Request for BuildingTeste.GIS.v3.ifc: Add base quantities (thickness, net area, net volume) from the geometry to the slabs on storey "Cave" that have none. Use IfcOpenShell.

First a look at what the model holds.

```python
import ifcopenshell
import ifcopenshell.util.element
import ifcopenshell.util.unit

model = ifcopenshell.open("BuildingTeste.GIS.v3.ifc")
print(model.schema)
for unit_type in ("LENGTHUNIT", "AREAUNIT", "VOLUMEUNIT"):
    print(unit_type, ifcopenshell.util.unit.calculate_unit_scale(model, unit_type))
storey = next(s for s in model.by_type("IfcBuildingStorey") if s.Name == "Cave")
slabs = [e for e in ifcopenshell.util.element.get_decomposition(storey) if e.is_a("IfcSlab")]
for e in sorted(slabs, key=lambda e: e.id()):
    print(e.id(), e.is_a(), e.Name, list(ifcopenshell.util.element.get_psets(e, qtos_only=True)), sep=" | ")
```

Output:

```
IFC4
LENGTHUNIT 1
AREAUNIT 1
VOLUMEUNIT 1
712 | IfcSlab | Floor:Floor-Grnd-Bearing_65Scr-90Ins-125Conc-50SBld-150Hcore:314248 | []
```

```python
import ifcopenshell
import ifcopenshell.api.pset
import ifcopenshell.geom
import ifcopenshell.util.element
import ifcopenshell.util.shape
import ifcopenshell.util.unit

model = ifcopenshell.open("BuildingTeste.GIS.v3.ifc")
unit_scale = ifcopenshell.util.unit.calculate_unit_scale(model)
area_scale = ifcopenshell.util.unit.calculate_unit_scale(model, "AREAUNIT")
volume_scale = ifcopenshell.util.unit.calculate_unit_scale(model, "VOLUMEUNIT")
settings = ifcopenshell.geom.settings()

storey = next(s for s in model.by_type("IfcBuildingStorey") if s.Name == "Cave")
slabs = [e for e in ifcopenshell.util.element.get_decomposition(storey) if e.is_a("IfcSlab")]

for e in sorted(slabs, key=lambda e: e.id()):
    if ifcopenshell.util.element.get_psets(e, qtos_only=True, should_inherit=False):
        continue
    # Geometry comes back in metres, in the element's own axes.
    shape = ifcopenshell.geom.create_shape(settings, e)
    values = {
        "Width": ifcopenshell.util.shape.get_z(shape.geometry) / unit_scale,
        "NetArea": ifcopenshell.util.shape.get_footprint_area(shape.geometry) / area_scale,
        "NetVolume": ifcopenshell.util.shape.get_volume(shape.geometry) / volume_scale,
    }
    qto = ifcopenshell.api.pset.add_qto(model, product=e, name="Qto_SlabBaseQuantities")
    ifcopenshell.api.pset.edit_qto(model, qto=qto, properties=values)
    print(e.id(), {k: round(v, 3) for k, v in values.items()})

model.write("BuildingTeste.GIS.v3_rev.ifc")
```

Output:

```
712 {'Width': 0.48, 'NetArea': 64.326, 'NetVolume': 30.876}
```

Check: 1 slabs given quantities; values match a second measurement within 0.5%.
